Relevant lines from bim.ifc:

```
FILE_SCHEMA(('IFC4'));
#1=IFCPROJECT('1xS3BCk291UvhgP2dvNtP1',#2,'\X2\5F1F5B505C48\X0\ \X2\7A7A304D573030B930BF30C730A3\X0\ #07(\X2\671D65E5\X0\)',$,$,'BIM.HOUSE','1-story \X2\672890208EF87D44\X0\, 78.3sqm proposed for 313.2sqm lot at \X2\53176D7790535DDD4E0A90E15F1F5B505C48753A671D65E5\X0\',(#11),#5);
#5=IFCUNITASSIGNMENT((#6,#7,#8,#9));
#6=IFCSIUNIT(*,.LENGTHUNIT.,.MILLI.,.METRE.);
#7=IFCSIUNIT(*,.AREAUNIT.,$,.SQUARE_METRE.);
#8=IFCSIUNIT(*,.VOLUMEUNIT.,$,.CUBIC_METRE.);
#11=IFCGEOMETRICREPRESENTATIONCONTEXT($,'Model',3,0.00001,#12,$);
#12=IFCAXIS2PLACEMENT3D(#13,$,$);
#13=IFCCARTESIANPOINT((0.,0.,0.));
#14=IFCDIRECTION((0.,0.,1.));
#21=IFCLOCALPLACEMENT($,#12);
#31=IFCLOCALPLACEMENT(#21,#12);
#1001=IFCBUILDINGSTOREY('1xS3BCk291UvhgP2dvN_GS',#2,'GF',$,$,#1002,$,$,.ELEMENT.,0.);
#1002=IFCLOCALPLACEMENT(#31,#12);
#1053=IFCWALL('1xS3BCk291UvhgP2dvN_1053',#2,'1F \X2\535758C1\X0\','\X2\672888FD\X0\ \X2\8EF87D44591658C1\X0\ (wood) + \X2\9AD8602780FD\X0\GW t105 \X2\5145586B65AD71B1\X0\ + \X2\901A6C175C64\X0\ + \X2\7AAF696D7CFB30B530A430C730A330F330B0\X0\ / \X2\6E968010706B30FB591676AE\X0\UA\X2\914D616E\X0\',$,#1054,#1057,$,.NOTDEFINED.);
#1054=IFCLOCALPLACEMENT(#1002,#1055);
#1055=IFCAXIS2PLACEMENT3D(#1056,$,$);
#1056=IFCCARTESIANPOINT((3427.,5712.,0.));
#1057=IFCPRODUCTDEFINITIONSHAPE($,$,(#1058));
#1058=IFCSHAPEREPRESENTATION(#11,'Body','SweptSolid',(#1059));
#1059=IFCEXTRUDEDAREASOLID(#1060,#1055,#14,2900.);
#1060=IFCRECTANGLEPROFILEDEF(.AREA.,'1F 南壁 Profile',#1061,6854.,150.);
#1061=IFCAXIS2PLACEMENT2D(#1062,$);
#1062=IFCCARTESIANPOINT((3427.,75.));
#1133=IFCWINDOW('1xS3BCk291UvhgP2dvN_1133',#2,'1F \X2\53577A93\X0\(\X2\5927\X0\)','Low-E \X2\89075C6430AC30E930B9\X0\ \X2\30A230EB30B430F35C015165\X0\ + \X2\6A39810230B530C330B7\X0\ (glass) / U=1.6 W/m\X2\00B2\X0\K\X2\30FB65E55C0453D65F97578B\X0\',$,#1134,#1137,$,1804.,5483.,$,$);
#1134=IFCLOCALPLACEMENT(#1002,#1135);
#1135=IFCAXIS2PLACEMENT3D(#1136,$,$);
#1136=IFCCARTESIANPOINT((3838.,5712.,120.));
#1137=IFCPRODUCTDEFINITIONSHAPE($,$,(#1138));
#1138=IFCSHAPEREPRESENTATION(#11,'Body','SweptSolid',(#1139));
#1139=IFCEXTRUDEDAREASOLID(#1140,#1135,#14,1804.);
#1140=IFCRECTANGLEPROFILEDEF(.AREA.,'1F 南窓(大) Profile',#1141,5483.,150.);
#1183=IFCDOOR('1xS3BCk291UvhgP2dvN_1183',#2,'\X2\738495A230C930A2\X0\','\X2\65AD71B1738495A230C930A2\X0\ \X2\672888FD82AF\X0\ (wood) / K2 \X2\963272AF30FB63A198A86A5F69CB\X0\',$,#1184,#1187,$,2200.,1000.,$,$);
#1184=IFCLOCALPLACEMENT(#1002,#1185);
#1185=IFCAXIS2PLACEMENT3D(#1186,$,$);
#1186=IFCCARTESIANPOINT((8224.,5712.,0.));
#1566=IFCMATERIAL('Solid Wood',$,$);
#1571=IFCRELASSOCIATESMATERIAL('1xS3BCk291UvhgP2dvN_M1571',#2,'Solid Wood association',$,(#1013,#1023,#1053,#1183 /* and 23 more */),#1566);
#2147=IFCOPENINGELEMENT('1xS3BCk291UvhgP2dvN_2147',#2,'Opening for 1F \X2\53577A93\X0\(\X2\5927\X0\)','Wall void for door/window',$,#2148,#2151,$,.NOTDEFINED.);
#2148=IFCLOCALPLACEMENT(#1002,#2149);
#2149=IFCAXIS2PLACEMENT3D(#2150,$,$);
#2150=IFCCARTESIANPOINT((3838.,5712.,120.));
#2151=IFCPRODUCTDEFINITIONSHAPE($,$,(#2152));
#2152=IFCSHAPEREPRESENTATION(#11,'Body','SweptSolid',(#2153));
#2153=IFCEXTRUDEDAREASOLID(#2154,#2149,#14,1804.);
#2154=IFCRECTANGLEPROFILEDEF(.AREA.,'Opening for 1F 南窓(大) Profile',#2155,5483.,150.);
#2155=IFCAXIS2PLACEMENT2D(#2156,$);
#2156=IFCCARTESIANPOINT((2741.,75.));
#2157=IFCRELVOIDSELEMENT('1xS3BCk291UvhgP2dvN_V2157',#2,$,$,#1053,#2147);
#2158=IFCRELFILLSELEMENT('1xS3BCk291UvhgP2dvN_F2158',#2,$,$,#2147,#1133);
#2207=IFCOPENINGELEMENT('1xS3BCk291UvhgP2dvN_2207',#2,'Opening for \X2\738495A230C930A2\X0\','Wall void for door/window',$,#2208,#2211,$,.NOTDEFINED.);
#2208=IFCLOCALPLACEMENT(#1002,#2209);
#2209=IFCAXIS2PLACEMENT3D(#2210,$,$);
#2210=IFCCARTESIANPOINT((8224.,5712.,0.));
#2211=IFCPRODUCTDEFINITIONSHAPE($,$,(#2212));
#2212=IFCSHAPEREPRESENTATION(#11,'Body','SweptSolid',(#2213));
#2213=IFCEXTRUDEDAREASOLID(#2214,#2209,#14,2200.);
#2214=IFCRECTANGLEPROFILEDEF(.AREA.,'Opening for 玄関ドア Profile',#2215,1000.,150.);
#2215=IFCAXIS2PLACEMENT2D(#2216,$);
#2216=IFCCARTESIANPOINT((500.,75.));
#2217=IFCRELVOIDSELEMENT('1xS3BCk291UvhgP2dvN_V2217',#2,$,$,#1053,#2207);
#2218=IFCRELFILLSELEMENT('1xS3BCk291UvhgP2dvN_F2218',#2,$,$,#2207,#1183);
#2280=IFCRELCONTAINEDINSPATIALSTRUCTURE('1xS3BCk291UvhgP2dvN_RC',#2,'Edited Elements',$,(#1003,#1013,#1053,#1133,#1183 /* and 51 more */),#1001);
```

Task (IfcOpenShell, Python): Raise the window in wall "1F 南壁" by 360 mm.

```python
import numpy as np
import ifcopenshell
import ifcopenshell.api.geometry
import ifcopenshell.util.placement
import ifcopenshell.util.unit

model = ifcopenshell.open("bim.ifc")
unit_scale = ifcopenshell.util.unit.calculate_unit_scale(model)

window = model.by_id(1133)
opening = window.FillsVoids[0].RelatingOpeningElement
dz = 360.0

shift = np.array([0.0, 0.0, dz])
# The window is not placed relative to its opening, so move both.
for product in (opening, window):
    matrix = ifcopenshell.util.placement.get_local_placement(product.ObjectPlacement)
    matrix[:3, 3] += shift
    ifcopenshell.api.geometry.edit_object_placement(model, product=product, matrix=matrix, is_si=False)

print(f"moved by {dz * unit_scale:+.3f} m")

model.write("bim_updated.ifc")
```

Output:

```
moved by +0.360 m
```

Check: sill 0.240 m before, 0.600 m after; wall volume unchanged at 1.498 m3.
